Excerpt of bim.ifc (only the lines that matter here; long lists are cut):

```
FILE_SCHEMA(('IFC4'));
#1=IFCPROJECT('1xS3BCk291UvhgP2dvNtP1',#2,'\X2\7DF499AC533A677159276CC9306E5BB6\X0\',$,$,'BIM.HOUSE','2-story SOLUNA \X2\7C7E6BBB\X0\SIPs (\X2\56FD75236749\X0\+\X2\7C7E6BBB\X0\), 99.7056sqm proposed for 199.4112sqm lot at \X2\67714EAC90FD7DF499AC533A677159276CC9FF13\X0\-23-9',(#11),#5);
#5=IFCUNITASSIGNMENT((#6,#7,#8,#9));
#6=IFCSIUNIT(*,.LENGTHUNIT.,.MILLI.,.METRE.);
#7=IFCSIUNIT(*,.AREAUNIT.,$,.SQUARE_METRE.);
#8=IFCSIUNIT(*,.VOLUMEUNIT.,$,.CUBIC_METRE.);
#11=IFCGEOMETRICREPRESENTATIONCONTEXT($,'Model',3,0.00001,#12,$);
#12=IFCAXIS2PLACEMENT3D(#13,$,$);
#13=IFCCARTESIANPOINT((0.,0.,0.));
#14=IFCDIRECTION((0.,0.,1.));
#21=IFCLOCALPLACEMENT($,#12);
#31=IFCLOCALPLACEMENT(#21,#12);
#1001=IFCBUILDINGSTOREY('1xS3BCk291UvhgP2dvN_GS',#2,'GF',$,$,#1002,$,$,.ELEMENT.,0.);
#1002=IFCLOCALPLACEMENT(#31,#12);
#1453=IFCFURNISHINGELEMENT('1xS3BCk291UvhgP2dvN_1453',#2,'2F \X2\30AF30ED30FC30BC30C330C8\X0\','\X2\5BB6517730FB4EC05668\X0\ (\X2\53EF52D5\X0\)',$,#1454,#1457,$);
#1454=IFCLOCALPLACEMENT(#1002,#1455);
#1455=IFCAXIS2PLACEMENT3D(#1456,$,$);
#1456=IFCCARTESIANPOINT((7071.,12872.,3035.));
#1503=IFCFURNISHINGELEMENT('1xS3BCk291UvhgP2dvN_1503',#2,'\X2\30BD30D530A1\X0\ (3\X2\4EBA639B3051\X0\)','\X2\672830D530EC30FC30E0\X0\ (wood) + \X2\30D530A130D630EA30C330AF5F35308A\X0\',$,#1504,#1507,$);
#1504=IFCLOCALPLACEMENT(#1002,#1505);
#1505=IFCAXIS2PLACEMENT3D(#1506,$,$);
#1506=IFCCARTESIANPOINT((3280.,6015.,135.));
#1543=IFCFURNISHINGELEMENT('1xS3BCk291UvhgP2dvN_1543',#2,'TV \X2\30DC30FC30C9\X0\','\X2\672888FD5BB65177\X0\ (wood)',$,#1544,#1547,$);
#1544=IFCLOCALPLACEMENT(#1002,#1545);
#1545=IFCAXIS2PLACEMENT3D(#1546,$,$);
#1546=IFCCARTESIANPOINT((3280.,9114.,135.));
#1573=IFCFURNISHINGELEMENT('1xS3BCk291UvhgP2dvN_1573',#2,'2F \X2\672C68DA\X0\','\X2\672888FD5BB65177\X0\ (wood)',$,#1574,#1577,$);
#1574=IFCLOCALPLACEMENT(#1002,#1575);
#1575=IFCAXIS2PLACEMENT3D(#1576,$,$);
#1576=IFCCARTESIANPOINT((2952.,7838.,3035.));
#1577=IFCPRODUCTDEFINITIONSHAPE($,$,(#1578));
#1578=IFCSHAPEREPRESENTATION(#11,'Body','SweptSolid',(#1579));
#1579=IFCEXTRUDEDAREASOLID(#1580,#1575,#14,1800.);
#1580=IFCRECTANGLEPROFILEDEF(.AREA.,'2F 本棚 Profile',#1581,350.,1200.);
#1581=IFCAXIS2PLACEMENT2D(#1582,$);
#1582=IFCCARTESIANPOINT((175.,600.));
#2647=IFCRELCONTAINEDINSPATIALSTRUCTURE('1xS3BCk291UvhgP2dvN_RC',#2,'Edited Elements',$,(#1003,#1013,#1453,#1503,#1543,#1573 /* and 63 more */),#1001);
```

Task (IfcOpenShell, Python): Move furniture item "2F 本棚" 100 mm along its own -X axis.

```python
import ifcopenshell
import ifcopenshell.api.geometry
import ifcopenshell.util.placement
import ifcopenshell.util.unit

model = ifcopenshell.open("bim.ifc")
unit_scale = ifcopenshell.util.unit.calculate_unit_scale(model)

item = model.by_guid("1xS3BCk291UvhgP2dvN_1573")
matrix = ifcopenshell.util.placement.get_local_placement(item.ObjectPlacement)
matrix[:3, 3] -= matrix[:3, 0] * 0.1 / unit_scale
ifcopenshell.api.geometry.edit_object_placement(model, product=item, matrix=matrix, is_si=False)

print(ifcopenshell.util.placement.get_local_placement(item.ObjectPlacement).round(3) + 0.0)

model.write("bim_v2.ifc")
```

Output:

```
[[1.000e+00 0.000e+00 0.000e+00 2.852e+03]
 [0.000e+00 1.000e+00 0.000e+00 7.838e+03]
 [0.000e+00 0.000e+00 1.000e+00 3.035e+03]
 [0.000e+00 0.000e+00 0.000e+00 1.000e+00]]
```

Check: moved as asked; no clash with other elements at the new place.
